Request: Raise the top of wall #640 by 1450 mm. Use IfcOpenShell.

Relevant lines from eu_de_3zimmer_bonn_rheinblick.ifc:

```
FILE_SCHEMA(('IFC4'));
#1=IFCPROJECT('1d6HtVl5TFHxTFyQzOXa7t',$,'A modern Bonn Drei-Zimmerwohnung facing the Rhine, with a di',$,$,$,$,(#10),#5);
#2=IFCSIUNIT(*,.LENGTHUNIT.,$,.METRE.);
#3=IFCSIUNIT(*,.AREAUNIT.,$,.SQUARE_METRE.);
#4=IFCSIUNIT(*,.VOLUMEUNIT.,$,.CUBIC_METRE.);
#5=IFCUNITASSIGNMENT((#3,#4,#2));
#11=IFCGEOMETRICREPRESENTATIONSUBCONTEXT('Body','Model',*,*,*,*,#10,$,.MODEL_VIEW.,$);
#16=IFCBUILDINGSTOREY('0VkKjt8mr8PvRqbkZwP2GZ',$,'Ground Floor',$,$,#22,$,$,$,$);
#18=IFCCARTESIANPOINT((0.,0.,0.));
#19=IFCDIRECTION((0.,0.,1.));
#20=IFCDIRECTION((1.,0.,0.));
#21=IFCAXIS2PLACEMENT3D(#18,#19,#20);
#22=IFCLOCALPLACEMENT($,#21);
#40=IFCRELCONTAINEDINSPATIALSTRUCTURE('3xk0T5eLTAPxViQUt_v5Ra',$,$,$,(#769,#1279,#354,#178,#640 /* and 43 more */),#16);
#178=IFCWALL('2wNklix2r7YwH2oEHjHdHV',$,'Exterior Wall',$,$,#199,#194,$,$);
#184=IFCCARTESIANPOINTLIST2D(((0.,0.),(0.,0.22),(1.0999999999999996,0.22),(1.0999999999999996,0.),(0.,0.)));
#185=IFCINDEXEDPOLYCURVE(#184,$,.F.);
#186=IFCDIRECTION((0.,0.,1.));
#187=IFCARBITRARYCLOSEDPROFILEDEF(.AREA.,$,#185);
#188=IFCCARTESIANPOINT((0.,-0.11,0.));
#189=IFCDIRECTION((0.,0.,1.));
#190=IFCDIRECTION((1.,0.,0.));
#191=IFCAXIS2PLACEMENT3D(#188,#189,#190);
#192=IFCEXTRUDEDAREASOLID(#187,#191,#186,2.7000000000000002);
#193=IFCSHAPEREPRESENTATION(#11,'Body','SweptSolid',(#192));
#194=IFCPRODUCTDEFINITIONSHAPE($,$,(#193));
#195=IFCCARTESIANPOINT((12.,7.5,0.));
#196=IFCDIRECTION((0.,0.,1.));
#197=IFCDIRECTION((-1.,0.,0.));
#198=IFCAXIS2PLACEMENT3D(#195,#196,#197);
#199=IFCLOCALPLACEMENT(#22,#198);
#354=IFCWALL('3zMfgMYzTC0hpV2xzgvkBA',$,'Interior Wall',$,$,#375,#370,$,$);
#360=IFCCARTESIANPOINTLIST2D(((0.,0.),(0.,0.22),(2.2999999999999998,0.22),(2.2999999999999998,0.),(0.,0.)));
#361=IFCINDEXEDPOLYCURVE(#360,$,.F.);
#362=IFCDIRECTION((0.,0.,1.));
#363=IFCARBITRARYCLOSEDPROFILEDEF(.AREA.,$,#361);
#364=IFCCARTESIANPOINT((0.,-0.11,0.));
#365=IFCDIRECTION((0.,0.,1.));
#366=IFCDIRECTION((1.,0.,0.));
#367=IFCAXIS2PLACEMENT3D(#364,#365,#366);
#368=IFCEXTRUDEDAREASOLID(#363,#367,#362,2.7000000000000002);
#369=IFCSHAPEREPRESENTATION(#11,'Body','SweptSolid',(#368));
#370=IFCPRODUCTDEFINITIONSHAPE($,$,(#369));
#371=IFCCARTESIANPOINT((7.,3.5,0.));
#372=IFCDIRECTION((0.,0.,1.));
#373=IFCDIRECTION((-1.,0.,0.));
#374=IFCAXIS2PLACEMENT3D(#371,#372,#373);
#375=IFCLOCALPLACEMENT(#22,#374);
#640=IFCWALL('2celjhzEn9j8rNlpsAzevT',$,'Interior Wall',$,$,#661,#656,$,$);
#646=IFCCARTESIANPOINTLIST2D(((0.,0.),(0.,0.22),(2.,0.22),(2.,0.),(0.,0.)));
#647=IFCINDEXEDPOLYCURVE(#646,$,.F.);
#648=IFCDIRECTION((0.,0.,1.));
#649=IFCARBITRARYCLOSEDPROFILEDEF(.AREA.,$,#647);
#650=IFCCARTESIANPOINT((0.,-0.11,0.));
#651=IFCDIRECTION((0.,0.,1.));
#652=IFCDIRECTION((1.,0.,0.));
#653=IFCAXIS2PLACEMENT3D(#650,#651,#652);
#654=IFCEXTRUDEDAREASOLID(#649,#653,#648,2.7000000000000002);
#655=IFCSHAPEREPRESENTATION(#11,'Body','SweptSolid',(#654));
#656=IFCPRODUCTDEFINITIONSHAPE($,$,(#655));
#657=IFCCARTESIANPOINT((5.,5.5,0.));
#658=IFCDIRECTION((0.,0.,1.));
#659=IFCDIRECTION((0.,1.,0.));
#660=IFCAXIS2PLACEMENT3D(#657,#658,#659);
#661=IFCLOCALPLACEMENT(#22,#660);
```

```python
import ifcopenshell
import ifcopenshell.geom
import ifcopenshell.util.representation
import ifcopenshell.util.shape

model = ifcopenshell.open("eu_de_3zimmer_bonn_rheinblick.ifc")
settings = ifcopenshell.geom.settings()


def volume(element):
    """Net volume in cubic metres, openings subtracted."""
    shape = ifcopenshell.geom.create_shape(settings, element)
    return ifcopenshell.util.shape.get_volume(shape.geometry)


wall = model.by_id(640)
before = volume(wall)

body = ifcopenshell.util.representation.get_representation(wall, "Model", "Body")
solid = body.Items[0]
old_height = solid.Depth
solid.Depth += 1.45
after = volume(wall)

print(f"height {old_height:g} -> {solid.Depth:g}, volume {before:.3f} -> {after:.3f} m3")

model.write("eu_de_3zimmer_bonn_rheinblick_rev.ifc")
```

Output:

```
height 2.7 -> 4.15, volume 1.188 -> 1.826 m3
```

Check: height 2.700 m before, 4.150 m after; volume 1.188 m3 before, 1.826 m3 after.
